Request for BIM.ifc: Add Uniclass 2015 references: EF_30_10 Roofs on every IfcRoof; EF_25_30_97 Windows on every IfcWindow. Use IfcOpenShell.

First a look at what the model holds.

```python
import ifcopenshell

model = ifcopenshell.open("BIM.ifc")
print(model.schema)
print("classifications:", [c.Name for c in model.by_type("IfcClassification")])
for ifc_class in ("IfcDoor", "IfcRoof", "IfcStair", "IfcWall", "IfcWindow"):
    print(ifc_class, len(model.by_type(ifc_class)))
```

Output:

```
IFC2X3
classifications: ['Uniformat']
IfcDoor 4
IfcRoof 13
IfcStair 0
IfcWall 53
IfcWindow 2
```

```python
import ifcopenshell
import ifcopenshell.api.classification

model = ifcopenshell.open("BIM.ifc")

# IFC2X3 requires Source and Edition and has no link from the project to the system.
system = model.create_entity("IfcClassification", Source="NBS", Edition="2015", Name="Uniclass 2015")

codes = {
    "IfcRoof": ("EF_30_10", "Roofs"),
    "IfcWindow": ("EF_25_30_97", "Windows"),
}
for ifc_class, (code, name) in codes.items():
    products = model.by_type(ifc_class)
    ifcopenshell.api.classification.add_reference(
        model, products=products, classification=system, identification=code, name=name
    )
    print(code, len(products))

model.write("BIM_rev.ifc")
```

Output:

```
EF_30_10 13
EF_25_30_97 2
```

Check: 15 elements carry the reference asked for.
